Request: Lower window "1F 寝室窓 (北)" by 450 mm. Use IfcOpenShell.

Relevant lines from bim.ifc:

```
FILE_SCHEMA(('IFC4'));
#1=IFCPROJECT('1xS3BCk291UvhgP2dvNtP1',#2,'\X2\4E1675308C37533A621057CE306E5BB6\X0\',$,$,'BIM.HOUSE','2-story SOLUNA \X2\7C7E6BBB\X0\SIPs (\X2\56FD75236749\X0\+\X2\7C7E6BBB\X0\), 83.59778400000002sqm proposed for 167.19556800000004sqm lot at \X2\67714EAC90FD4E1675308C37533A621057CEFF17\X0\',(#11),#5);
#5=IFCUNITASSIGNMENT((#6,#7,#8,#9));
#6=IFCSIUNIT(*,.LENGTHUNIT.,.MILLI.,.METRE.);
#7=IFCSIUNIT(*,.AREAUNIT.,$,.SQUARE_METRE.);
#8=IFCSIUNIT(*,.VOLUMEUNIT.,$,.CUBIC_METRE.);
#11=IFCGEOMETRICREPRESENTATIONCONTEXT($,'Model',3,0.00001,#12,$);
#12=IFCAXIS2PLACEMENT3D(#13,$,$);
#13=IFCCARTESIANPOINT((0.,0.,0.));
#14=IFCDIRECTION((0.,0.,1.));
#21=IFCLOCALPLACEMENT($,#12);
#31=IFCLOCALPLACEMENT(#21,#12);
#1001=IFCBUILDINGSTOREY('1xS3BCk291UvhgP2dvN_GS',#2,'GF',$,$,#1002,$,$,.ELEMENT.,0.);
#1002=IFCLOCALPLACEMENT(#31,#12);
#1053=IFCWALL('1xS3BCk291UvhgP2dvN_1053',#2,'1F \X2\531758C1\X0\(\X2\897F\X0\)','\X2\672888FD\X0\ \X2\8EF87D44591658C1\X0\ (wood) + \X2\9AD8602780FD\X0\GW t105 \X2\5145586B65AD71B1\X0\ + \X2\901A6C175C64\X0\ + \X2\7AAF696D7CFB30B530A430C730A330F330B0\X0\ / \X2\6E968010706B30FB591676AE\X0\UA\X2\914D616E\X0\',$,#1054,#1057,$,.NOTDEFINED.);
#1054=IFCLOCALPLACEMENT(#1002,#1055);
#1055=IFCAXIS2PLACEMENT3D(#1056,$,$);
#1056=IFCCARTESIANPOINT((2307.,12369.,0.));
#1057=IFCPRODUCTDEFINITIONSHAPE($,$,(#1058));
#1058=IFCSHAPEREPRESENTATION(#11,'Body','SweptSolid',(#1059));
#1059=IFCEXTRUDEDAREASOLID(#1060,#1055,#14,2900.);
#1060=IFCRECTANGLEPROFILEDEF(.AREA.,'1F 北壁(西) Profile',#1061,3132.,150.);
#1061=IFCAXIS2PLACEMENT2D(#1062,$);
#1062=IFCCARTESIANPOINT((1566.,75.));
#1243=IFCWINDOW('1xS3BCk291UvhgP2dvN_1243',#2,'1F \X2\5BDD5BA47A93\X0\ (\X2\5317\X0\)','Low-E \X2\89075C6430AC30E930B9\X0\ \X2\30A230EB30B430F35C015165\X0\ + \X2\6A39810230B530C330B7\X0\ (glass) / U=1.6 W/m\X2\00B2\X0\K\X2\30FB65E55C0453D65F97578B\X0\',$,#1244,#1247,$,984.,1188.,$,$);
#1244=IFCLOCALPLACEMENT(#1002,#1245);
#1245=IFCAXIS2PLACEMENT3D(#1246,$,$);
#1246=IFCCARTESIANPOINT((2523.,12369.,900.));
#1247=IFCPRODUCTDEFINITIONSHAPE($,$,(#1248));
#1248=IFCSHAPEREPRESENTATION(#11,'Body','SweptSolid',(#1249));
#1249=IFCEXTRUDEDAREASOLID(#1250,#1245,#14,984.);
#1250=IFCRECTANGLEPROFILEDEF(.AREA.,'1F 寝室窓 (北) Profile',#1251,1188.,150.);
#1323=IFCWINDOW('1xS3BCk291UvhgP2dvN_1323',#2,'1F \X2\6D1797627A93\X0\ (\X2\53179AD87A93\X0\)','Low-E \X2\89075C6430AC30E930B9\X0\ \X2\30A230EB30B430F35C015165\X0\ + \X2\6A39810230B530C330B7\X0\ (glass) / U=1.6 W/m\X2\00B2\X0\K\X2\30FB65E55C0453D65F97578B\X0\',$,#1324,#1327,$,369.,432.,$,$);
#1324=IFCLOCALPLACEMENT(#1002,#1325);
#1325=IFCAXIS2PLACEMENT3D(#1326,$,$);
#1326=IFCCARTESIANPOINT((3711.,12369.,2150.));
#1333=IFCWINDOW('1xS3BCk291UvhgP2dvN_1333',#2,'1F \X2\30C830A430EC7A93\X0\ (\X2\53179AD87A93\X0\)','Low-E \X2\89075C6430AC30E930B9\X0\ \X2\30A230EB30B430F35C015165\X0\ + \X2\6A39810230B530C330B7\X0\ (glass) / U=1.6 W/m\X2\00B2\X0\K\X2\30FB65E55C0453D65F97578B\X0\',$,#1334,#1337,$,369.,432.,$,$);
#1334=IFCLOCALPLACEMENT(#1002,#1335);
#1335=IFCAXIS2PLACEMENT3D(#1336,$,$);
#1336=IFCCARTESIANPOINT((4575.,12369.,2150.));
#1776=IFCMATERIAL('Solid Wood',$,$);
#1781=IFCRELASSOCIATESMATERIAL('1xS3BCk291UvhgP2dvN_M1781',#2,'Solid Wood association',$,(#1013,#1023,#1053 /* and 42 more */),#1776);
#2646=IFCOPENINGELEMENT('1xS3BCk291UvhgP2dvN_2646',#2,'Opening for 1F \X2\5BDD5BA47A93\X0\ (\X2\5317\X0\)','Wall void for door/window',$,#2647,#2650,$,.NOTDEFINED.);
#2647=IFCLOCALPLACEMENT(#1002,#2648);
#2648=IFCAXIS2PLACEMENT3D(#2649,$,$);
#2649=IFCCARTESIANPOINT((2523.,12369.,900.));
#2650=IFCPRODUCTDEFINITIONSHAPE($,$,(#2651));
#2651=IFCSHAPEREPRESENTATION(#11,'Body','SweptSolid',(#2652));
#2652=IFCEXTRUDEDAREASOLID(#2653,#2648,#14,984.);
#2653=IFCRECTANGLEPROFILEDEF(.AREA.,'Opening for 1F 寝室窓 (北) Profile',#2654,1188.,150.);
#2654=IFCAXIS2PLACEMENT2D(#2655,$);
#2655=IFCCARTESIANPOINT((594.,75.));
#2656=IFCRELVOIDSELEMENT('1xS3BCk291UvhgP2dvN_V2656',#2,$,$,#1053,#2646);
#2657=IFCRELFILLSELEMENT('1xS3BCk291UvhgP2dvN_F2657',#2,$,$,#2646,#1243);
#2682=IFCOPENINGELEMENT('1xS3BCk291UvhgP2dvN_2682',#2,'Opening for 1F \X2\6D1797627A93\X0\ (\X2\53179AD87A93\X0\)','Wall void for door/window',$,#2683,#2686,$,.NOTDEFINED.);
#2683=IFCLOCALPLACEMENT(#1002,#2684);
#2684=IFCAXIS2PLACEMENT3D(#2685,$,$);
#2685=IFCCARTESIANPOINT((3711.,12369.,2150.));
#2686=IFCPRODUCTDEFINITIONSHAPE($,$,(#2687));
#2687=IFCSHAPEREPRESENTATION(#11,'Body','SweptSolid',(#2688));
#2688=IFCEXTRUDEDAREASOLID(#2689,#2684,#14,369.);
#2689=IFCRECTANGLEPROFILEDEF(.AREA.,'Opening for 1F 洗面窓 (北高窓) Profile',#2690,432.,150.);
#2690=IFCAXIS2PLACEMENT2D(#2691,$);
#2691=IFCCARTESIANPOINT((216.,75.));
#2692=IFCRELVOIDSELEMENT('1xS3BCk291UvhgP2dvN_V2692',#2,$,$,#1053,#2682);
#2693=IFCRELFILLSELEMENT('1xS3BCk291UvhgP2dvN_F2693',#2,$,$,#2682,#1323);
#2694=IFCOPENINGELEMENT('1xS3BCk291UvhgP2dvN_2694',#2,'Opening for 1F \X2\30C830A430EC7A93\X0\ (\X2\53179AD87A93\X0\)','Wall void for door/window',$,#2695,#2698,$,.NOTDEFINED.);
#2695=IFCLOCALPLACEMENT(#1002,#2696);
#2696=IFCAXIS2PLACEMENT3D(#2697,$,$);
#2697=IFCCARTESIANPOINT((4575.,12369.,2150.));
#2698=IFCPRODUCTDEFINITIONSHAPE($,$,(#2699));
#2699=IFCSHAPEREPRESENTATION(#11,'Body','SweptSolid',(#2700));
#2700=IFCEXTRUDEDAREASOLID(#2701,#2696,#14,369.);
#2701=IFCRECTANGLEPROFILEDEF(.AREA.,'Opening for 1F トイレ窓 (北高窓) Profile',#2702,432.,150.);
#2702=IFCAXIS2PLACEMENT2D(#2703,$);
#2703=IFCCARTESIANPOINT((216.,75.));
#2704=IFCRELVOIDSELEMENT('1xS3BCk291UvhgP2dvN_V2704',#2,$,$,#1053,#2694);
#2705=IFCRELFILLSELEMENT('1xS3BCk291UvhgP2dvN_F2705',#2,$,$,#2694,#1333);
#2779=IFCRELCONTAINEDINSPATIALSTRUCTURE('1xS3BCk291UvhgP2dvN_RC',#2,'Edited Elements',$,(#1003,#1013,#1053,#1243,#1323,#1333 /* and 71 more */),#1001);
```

```python
import numpy as np
import ifcopenshell
import ifcopenshell.api.geometry
import ifcopenshell.util.placement
import ifcopenshell.util.unit

model = ifcopenshell.open("bim.ifc")
unit_scale = ifcopenshell.util.unit.calculate_unit_scale(model)

window = model.by_guid("1xS3BCk291UvhgP2dvN_1243")
opening = window.FillsVoids[0].RelatingOpeningElement
dz = -0.45 / unit_scale

shift = np.array([0.0, 0.0, dz])
# The window is not placed relative to its opening, so move both.
for product in (opening, window):
    matrix = ifcopenshell.util.placement.get_local_placement(product.ObjectPlacement)
    matrix[:3, 3] += shift
    ifcopenshell.api.geometry.edit_object_placement(model, product=product, matrix=matrix, is_si=False)

print(f"moved by {dz * unit_scale:+.3f} m")

model.write("bim_updated.ifc")
```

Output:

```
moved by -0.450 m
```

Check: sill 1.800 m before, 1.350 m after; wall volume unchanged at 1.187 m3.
